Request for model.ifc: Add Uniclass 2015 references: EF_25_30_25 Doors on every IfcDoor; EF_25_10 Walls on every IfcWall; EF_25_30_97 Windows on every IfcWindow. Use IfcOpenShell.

First a look at what the model holds.

```python
import ifcopenshell

model = ifcopenshell.open("model.ifc")
print(model.schema)
print("classifications:", [c.Name for c in model.by_type("IfcClassification")])
for ifc_class in ("IfcDoor", "IfcRoof", "IfcStair", "IfcWall", "IfcWindow"):
    print(ifc_class, len(model.by_type(ifc_class)))
```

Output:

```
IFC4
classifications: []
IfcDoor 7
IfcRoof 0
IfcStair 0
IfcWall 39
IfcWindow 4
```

```python
import ifcopenshell
import ifcopenshell.api.classification

model = ifcopenshell.open("model.ifc")

system = ifcopenshell.api.classification.add_classification(model, classification="Uniclass 2015")

codes = {
    "IfcDoor": ("EF_25_30_25", "Doors"),
    "IfcWall": ("EF_25_10", "Walls"),
    "IfcWindow": ("EF_25_30_97", "Windows"),
}
for ifc_class, (code, name) in codes.items():
    products = model.by_type(ifc_class)
    ifcopenshell.api.classification.add_reference(
        model, products=products, classification=system, identification=code, name=name
    )
    print(code, len(products))

model.write("model-out.ifc")
```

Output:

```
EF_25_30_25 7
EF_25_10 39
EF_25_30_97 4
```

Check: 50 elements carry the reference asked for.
